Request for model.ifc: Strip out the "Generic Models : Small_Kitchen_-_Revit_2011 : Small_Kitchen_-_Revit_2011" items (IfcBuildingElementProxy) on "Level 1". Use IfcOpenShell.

First a look at what the model holds.

```python
import ifcopenshell
import ifcopenshell.util.element

model = ifcopenshell.open("model.ifc")
print(model.schema)
storey = next(s for s in model.by_type("IfcBuildingStorey") if s.Name == "Level 1")
proxies = [e for e in ifcopenshell.util.element.get_decomposition(storey) if e.is_a("IfcBuildingElementProxy")]
seen = {}
for e in proxies:
    element_type = ifcopenshell.util.element.get_type(e)
    name = element_type.Name if element_type not in (None, e) else None
    seen[name] = seen.get(name, 0) + 1
for name, count in sorted(seen.items(), key=str):
    print(count, "x", name)
```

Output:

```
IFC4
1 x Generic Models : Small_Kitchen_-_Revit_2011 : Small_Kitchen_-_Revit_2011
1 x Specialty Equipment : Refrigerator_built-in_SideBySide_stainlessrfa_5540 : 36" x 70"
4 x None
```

```python
import ifcopenshell
import ifcopenshell.api.root
import ifcopenshell.util.element

model = ifcopenshell.open("model.ifc")

storey = next(s for s in model.by_type("IfcBuildingStorey") if s.Name == "Level 1")
proxies = [e for e in ifcopenshell.util.element.get_decomposition(storey) if e.is_a("IfcBuildingElementProxy")]
targets = [e for e in proxies if (t := ifcopenshell.util.element.get_type(e)) not in (None, e) and t.Name == "Generic Models : Small_Kitchen_-_Revit_2011 : Small_Kitchen_-_Revit_2011"]

for e in targets:
    ifcopenshell.api.root.remove_product(model, product=e)
print(len(targets), "removed")

model.write("model_edited.ifc")
```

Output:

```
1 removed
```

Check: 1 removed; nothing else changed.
